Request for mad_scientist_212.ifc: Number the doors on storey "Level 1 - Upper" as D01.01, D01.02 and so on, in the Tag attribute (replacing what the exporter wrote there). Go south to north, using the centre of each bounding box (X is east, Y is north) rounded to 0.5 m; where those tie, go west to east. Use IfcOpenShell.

First a look at what the model holds.

```python
import ifcopenshell
import ifcopenshell.util.element
import ifcopenshell.util.placement

model = ifcopenshell.open("mad_scientist_212.ifc")
print(model.schema)
storey = next(s for s in model.by_type("IfcBuildingStorey") if s.Name == "Level 1 - Upper")
doors = [e for e in ifcopenshell.util.element.get_decomposition(storey) if e.is_a("IfcDoor")]
for e in sorted(doors, key=lambda e: e.id()):
    origin = ifcopenshell.util.placement.get_local_placement(e.ObjectPlacement)[:3, 3]
    print(e.id(), e.Tag, e.Name, origin.round(2) + 0.0, sep=" | ")
```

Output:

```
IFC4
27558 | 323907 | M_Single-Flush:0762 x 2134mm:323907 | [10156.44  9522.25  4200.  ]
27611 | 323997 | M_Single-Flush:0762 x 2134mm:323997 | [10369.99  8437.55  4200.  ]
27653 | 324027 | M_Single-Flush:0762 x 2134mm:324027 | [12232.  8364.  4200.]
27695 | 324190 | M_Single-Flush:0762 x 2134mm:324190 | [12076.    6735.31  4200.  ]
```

```python
import ifcopenshell
import ifcopenshell.geom
import ifcopenshell.util.element
import ifcopenshell.util.shape

model = ifcopenshell.open("mad_scientist_212.ifc")
settings = ifcopenshell.geom.settings()
settings.set("use-world-coords", True)


def centre(element):
    shape = ifcopenshell.geom.create_shape(settings, element)
    return ifcopenshell.util.shape.get_bbox_centroid(shape.geometry)


storey = next(s for s in model.by_type("IfcBuildingStorey") if s.Name == "Level 1 - Upper")
doors = [e for e in ifcopenshell.util.element.get_decomposition(storey) if e.is_a("IfcDoor")]

# Insertion points can sit at a corner or the storey origin, so sort by the geometry (in metres).
centres = {e: centre(e) for e in doors}
doors.sort(key=lambda e: (round(centres[e][1] / 0.5), centres[e][0]))

for i, e in enumerate(doors, start=1):
    number = f"D01.{i:02d}"
    e.Tag = number
    print(e.id(), number)

model.write("mad_scientist_212-out.ifc")
```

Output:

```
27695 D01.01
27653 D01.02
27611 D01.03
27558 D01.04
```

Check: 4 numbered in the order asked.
